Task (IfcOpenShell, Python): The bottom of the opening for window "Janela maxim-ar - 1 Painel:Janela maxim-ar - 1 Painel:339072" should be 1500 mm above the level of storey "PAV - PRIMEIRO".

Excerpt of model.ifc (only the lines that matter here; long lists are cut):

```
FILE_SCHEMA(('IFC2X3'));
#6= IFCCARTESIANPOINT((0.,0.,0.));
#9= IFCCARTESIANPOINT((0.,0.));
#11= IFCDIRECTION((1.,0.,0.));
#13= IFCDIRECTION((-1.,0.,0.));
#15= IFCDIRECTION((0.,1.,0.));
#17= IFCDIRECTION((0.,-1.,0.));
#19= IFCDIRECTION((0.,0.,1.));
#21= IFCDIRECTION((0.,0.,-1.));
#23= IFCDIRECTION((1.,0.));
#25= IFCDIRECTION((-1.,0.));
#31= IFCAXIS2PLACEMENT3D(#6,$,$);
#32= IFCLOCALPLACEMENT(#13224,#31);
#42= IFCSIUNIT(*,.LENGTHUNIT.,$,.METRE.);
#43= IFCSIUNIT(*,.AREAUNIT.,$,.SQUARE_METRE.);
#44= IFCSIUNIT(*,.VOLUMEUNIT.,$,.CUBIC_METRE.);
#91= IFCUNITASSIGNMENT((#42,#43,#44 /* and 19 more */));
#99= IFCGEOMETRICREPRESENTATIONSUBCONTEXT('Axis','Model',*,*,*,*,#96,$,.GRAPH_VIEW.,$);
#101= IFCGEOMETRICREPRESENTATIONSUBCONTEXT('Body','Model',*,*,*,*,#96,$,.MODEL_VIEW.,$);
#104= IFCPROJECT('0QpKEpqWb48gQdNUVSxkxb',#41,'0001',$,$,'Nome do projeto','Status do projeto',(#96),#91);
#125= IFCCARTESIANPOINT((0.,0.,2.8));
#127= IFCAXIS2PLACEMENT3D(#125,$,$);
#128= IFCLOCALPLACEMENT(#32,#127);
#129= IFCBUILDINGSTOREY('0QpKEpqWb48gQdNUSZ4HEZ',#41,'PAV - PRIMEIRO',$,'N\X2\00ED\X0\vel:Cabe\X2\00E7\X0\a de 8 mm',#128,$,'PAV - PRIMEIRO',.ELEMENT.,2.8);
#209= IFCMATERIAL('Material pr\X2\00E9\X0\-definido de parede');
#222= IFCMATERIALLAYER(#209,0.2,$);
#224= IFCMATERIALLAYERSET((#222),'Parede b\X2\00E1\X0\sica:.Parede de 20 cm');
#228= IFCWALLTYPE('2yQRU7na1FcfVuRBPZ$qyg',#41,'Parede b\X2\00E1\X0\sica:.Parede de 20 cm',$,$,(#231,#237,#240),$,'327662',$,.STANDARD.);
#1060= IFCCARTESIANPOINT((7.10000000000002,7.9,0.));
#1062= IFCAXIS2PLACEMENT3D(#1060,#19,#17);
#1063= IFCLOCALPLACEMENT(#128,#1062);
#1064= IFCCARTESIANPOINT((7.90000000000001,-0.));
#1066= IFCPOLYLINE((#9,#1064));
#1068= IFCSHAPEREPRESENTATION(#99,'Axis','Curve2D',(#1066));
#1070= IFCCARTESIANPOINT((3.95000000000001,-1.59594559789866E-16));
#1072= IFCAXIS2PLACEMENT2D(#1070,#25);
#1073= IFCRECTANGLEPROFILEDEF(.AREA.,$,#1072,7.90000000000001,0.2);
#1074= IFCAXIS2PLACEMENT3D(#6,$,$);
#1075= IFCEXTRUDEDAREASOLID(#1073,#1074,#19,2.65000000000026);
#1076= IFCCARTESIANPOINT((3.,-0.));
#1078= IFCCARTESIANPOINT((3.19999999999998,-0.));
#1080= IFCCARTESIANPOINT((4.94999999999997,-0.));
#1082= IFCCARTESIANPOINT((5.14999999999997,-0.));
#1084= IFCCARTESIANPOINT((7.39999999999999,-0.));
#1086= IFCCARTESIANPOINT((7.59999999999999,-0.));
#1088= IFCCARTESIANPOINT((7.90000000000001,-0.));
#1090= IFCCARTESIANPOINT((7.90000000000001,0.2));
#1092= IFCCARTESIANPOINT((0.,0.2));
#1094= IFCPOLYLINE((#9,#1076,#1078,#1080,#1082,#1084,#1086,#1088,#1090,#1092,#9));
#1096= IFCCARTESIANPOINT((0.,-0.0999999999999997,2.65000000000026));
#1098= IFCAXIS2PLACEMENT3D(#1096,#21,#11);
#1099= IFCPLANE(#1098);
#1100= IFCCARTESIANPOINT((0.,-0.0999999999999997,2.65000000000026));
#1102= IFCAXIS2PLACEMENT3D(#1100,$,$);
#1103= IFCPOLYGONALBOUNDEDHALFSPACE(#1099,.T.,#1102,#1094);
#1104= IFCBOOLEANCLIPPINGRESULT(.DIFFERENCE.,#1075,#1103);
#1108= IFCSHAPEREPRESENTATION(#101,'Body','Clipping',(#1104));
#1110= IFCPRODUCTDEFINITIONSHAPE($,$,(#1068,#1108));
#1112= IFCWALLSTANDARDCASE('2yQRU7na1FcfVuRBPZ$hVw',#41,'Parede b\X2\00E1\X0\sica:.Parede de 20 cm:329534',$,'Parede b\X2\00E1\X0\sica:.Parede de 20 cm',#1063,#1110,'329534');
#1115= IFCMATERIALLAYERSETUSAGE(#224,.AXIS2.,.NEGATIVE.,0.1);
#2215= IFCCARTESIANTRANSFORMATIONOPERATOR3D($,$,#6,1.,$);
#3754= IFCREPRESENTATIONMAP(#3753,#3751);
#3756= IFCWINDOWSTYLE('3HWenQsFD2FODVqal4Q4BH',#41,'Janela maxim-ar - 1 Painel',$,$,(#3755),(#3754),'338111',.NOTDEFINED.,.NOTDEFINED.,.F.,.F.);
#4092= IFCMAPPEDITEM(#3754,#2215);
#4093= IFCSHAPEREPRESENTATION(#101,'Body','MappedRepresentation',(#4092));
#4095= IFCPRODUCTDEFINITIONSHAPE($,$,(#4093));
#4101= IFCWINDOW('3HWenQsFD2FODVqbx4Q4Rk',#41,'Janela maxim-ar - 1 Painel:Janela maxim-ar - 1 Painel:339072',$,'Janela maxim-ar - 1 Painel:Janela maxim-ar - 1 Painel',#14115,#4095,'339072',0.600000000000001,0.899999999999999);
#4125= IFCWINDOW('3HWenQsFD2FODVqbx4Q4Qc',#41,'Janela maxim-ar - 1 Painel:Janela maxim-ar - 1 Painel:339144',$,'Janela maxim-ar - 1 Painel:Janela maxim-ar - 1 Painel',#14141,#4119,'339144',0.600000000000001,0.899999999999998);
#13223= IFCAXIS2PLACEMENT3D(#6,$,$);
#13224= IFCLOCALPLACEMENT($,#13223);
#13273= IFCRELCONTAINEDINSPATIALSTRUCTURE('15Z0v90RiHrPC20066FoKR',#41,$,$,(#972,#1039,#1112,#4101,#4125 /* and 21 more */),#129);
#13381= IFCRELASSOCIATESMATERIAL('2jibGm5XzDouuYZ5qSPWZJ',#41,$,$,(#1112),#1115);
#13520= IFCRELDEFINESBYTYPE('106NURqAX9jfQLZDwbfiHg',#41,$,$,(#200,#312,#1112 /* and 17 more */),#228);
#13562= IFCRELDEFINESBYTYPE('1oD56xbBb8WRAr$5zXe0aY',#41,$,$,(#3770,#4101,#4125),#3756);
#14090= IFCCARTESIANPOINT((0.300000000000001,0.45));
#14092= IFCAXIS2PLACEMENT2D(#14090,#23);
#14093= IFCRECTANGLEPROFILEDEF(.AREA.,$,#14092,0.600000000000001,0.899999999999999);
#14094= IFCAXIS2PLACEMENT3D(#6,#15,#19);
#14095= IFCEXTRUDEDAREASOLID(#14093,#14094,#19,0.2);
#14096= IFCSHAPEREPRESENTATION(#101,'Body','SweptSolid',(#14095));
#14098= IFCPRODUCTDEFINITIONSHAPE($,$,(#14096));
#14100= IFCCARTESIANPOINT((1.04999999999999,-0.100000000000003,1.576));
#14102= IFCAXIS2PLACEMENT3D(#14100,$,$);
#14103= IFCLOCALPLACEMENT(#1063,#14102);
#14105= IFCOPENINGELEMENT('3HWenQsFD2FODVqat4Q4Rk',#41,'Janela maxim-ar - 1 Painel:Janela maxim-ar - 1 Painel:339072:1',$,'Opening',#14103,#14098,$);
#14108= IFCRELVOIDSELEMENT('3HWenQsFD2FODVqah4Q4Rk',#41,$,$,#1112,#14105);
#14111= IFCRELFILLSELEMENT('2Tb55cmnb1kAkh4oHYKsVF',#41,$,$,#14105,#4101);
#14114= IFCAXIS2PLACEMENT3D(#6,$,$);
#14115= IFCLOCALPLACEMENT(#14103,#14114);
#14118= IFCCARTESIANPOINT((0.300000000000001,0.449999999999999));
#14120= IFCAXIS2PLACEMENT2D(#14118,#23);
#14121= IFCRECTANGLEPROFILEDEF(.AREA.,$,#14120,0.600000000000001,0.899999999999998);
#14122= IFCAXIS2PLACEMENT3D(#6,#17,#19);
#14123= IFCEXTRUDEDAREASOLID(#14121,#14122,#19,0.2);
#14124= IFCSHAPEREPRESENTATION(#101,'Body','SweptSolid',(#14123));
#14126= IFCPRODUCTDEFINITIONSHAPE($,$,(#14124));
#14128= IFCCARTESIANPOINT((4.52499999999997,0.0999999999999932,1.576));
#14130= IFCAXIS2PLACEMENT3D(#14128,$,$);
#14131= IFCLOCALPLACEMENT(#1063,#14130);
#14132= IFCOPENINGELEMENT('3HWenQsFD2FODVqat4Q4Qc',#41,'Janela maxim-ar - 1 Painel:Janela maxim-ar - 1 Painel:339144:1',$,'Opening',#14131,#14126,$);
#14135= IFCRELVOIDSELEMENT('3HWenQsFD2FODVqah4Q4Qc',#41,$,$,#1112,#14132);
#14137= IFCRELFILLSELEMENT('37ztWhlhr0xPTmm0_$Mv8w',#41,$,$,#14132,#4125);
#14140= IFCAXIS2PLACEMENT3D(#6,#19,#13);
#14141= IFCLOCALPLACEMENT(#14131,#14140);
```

```python
import numpy as np
import ifcopenshell
import ifcopenshell.api.geometry
import ifcopenshell.geom
import ifcopenshell.util.element
import ifcopenshell.util.placement
import ifcopenshell.util.shape
import ifcopenshell.util.unit

model = ifcopenshell.open("model.ifc")
unit_scale = ifcopenshell.util.unit.calculate_unit_scale(model)

window = model.by_guid("3HWenQsFD2FODVqbx4Q4Rk")
opening = window.FillsVoids[0].RelatingOpeningElement
storey = ifcopenshell.util.element.get_container(window, ifc_class="IfcBuildingStorey")
level = ifcopenshell.util.placement.get_local_placement(storey.ObjectPlacement)[2, 3]

# The opening's origin need not be at the sill, so measure its lowest point.
shape = ifcopenshell.geom.create_shape(ifcopenshell.geom.settings(), opening)
bottom = ifcopenshell.util.shape.get_shape_bottom_elevation(shape, shape.geometry) / unit_scale
dz = level + 1.5 - bottom

shift = np.array([0.0, 0.0, dz])
# The window is placed relative to its opening, so it follows when the opening moves.
matrix = ifcopenshell.util.placement.get_local_placement(opening.ObjectPlacement)
matrix[:3, 3] += shift
ifcopenshell.api.geometry.edit_object_placement(
    model, product=opening, matrix=matrix, is_si=False, should_transform_children=True
)

print(f"moved by {dz * unit_scale:+.3f} m")

model.write("model-out.ifc")
```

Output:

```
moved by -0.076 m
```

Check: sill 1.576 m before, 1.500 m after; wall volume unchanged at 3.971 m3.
